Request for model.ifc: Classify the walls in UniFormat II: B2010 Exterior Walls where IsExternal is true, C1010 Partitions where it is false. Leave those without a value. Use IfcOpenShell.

First a look at what the model holds.

```python
import ifcopenshell
import ifcopenshell.util.element

model = ifcopenshell.open("model.ifc")
print(model.schema)
print("classifications:", [c.Name for c in model.by_type("IfcClassification")])
values = [ifcopenshell.util.element.get_pset(e, "Pset_WallCommon", "IsExternal") for e in model.by_type("IfcWall")]
for value in (True, False, None):
    print("IsExternal", value, values.count(value))
```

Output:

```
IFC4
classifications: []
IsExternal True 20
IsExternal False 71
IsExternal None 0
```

```python
import ifcopenshell
import ifcopenshell.api.classification
import ifcopenshell.util.element

model = ifcopenshell.open("model.ifc")

system = ifcopenshell.api.classification.add_classification(model, classification="UniFormat II")

walls = model.by_type("IfcWall")
external = {e: ifcopenshell.util.element.get_pset(e, "Pset_WallCommon", "IsExternal") for e in walls}
for flag, code, name in ((True, "B2010", "Exterior Walls"), (False, "C1010", "Partitions")):
    products = [e for e in walls if external[e] is flag]
    ifcopenshell.api.classification.add_reference(
        model, products=products, classification=system, identification=code, name=name
    )
    print(code, len(products))

model.write("model_rev.ifc")
```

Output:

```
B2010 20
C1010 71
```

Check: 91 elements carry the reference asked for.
